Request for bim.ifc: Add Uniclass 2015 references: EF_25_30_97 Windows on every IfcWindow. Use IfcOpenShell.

First a look at what the model holds.

```python
import ifcopenshell

model = ifcopenshell.open("bim.ifc")
print(model.schema)
print("classifications:", [c.Name for c in model.by_type("IfcClassification")])
for ifc_class in ("IfcDoor", "IfcRoof", "IfcStair", "IfcWall", "IfcWindow"):
    print(ifc_class, len(model.by_type(ifc_class)))
```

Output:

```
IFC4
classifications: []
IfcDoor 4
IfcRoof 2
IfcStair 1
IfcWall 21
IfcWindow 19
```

```python
import ifcopenshell
import ifcopenshell.api.classification

model = ifcopenshell.open("bim.ifc")

system = ifcopenshell.api.classification.add_classification(model, classification="Uniclass 2015")

codes = {
    "IfcWindow": ("EF_25_30_97", "Windows"),
}
for ifc_class, (code, name) in codes.items():
    products = model.by_type(ifc_class)
    ifcopenshell.api.classification.add_reference(
        model, products=products, classification=system, identification=code, name=name
    )
    print(code, len(products))

model.write("bim_edited.ifc")
```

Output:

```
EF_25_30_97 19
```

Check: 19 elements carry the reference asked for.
